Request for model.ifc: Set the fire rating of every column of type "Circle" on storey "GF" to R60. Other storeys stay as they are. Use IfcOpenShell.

First a look at what the model holds.

```python
import ifcopenshell
import ifcopenshell.util.element

model = ifcopenshell.open("model.ifc")
print(model.schema)
storey = next(s for s in model.by_type("IfcBuildingStorey") if s.Name == "GF")
columns = [e for e in ifcopenshell.util.element.get_decomposition(storey) if e.is_a("IfcColumn")]
seen = {}
for e in columns:
    element_type = ifcopenshell.util.element.get_type(e)
    key = (element_type.Name if element_type != e and element_type else None, ifcopenshell.util.element.get_pset(e, "Pset_ColumnCommon", "FireRating"))
    seen[key] = seen.get(key, 0) + 1
for (name, value), count in sorted(seen.items(), key=str):
    print(count, "x", name, "|", value)
```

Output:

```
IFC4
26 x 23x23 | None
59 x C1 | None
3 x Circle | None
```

```python
import ifcopenshell
import ifcopenshell.api.pset
import ifcopenshell.util.element

model = ifcopenshell.open("model.ifc")

storey = next(s for s in model.by_type("IfcBuildingStorey") if s.Name == "GF")
columns = [e for e in ifcopenshell.util.element.get_decomposition(storey) if e.is_a("IfcColumn")]

count = 0
for e in columns:
    element_type = ifcopenshell.util.element.get_type(e)
    if element_type in (None, e) or element_type.Name != "Circle":
        continue
    # add_pset returns the element's existing set when there is one.
    pset = ifcopenshell.api.pset.add_pset(model, product=e, name="Pset_ColumnCommon")
    ifcopenshell.api.pset.edit_pset(model, pset=pset, properties={"FireRating": "R60"})
    count += 1

print(count, "columns updated")

model.write("model_edited.ifc")
```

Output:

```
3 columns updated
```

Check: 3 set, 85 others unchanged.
